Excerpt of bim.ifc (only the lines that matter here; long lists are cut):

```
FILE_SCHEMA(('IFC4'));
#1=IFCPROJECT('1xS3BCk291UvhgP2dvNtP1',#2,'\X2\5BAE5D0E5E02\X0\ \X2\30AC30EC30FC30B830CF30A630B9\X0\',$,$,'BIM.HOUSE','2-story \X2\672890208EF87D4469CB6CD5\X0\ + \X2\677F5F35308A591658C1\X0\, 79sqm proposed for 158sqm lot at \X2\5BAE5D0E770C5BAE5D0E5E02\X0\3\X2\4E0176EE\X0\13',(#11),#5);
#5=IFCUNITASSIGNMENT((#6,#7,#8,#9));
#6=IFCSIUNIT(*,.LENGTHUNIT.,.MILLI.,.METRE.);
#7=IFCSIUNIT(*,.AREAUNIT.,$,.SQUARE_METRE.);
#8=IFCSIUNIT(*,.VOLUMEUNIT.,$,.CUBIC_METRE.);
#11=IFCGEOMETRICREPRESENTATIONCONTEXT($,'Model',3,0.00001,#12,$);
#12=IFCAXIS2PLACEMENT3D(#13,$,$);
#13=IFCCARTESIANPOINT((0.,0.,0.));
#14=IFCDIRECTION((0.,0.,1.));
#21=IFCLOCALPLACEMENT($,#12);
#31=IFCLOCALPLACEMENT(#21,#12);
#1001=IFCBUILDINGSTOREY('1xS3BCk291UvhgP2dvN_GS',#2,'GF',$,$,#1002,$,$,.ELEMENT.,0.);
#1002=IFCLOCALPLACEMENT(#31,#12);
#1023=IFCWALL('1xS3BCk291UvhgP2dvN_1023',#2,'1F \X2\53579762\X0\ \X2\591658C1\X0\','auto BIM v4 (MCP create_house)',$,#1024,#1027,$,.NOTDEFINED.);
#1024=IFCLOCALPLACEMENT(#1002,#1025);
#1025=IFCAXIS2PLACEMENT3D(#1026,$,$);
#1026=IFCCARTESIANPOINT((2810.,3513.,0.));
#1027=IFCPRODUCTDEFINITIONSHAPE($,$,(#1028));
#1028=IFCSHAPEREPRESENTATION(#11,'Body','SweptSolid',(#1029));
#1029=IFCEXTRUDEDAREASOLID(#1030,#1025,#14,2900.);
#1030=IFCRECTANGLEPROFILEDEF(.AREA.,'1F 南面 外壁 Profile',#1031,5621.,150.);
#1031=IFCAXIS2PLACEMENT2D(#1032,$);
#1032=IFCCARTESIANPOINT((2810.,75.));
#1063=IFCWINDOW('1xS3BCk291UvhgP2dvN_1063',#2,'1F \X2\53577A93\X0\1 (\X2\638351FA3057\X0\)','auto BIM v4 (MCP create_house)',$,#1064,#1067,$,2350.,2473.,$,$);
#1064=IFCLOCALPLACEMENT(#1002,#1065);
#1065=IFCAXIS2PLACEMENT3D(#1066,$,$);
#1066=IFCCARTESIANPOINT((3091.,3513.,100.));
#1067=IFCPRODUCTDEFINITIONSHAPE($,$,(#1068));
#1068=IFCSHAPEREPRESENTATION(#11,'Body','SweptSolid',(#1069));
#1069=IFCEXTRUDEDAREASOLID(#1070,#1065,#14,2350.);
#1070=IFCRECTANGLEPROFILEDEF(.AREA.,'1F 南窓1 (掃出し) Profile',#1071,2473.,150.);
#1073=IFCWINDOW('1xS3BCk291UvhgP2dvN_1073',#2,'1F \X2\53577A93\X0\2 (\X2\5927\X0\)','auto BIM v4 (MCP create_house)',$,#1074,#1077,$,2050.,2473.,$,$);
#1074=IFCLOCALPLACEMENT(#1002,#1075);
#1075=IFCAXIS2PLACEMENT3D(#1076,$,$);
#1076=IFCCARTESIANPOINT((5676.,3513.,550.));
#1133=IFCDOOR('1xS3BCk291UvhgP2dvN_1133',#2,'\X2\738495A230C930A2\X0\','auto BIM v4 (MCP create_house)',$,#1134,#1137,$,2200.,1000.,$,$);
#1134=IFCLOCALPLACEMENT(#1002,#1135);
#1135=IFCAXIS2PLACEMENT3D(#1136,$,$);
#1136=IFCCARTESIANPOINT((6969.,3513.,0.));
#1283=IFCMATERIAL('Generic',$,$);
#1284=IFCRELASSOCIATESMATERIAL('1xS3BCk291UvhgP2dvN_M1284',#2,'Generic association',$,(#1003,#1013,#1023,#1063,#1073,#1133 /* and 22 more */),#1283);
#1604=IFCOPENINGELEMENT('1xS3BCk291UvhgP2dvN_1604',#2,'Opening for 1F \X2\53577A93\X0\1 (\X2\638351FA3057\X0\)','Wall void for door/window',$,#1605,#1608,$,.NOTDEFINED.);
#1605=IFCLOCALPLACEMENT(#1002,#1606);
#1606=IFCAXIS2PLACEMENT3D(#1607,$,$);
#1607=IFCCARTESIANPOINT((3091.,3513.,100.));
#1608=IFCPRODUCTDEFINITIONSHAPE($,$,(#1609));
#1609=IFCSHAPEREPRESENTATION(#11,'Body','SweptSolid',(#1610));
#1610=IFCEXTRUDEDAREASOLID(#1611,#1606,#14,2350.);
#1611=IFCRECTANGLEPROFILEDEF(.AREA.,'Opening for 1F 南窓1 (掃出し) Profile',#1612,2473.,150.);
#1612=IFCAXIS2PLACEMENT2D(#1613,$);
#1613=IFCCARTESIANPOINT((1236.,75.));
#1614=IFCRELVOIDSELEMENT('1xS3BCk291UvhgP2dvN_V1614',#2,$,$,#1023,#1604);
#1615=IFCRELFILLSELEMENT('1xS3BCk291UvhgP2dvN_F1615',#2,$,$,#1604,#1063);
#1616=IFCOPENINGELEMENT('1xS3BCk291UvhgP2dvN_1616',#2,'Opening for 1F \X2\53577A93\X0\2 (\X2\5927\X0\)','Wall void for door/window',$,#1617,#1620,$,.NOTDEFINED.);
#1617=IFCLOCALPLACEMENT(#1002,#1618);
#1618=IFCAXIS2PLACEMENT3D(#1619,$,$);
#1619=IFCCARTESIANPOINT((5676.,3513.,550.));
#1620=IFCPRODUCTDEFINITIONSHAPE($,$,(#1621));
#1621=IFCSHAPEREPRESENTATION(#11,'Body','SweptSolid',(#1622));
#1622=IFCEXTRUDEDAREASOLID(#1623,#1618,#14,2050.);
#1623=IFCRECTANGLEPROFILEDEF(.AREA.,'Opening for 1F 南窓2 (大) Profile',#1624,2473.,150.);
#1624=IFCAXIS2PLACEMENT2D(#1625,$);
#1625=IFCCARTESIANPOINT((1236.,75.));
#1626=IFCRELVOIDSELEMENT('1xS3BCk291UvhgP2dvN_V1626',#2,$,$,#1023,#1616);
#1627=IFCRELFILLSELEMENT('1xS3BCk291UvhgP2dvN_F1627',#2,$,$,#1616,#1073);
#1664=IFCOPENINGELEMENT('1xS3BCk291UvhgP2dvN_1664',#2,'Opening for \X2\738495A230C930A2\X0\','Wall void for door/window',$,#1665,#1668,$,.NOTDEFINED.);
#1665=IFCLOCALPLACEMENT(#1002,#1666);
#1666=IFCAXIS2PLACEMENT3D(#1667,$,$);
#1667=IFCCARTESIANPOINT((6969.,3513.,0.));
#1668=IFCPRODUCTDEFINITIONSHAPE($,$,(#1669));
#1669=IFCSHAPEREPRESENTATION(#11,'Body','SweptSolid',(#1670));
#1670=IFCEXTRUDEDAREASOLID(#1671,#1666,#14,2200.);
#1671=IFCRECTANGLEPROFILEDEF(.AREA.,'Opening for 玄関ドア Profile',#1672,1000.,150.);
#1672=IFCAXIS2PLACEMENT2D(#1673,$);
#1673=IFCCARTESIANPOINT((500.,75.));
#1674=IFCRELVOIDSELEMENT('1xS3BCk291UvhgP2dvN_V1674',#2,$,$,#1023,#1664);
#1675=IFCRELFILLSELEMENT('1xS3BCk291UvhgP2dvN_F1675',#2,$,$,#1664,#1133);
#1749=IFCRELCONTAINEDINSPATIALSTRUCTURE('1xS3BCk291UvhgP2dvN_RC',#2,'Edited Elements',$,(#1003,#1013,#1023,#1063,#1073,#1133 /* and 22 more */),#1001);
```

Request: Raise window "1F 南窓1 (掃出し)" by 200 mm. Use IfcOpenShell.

```python
import numpy as np
import ifcopenshell
import ifcopenshell.api.geometry
import ifcopenshell.util.placement
import ifcopenshell.util.unit

model = ifcopenshell.open("bim.ifc")
unit_scale = ifcopenshell.util.unit.calculate_unit_scale(model)

window = model.by_guid("1xS3BCk291UvhgP2dvN_1063")
opening = window.FillsVoids[0].RelatingOpeningElement
dz = 0.2 / unit_scale

shift = np.array([0.0, 0.0, dz])
# The window is not placed relative to its opening, so move both.
for product in (opening, window):
    matrix = ifcopenshell.util.placement.get_local_placement(product.ObjectPlacement)
    matrix[:3, 3] += shift
    ifcopenshell.api.geometry.edit_object_placement(model, product=product, matrix=matrix, is_si=False)

print(f"moved by {dz * unit_scale:+.3f} m")

model.write("bim_edited.ifc")
```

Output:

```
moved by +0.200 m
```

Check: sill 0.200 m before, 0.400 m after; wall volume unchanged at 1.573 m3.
